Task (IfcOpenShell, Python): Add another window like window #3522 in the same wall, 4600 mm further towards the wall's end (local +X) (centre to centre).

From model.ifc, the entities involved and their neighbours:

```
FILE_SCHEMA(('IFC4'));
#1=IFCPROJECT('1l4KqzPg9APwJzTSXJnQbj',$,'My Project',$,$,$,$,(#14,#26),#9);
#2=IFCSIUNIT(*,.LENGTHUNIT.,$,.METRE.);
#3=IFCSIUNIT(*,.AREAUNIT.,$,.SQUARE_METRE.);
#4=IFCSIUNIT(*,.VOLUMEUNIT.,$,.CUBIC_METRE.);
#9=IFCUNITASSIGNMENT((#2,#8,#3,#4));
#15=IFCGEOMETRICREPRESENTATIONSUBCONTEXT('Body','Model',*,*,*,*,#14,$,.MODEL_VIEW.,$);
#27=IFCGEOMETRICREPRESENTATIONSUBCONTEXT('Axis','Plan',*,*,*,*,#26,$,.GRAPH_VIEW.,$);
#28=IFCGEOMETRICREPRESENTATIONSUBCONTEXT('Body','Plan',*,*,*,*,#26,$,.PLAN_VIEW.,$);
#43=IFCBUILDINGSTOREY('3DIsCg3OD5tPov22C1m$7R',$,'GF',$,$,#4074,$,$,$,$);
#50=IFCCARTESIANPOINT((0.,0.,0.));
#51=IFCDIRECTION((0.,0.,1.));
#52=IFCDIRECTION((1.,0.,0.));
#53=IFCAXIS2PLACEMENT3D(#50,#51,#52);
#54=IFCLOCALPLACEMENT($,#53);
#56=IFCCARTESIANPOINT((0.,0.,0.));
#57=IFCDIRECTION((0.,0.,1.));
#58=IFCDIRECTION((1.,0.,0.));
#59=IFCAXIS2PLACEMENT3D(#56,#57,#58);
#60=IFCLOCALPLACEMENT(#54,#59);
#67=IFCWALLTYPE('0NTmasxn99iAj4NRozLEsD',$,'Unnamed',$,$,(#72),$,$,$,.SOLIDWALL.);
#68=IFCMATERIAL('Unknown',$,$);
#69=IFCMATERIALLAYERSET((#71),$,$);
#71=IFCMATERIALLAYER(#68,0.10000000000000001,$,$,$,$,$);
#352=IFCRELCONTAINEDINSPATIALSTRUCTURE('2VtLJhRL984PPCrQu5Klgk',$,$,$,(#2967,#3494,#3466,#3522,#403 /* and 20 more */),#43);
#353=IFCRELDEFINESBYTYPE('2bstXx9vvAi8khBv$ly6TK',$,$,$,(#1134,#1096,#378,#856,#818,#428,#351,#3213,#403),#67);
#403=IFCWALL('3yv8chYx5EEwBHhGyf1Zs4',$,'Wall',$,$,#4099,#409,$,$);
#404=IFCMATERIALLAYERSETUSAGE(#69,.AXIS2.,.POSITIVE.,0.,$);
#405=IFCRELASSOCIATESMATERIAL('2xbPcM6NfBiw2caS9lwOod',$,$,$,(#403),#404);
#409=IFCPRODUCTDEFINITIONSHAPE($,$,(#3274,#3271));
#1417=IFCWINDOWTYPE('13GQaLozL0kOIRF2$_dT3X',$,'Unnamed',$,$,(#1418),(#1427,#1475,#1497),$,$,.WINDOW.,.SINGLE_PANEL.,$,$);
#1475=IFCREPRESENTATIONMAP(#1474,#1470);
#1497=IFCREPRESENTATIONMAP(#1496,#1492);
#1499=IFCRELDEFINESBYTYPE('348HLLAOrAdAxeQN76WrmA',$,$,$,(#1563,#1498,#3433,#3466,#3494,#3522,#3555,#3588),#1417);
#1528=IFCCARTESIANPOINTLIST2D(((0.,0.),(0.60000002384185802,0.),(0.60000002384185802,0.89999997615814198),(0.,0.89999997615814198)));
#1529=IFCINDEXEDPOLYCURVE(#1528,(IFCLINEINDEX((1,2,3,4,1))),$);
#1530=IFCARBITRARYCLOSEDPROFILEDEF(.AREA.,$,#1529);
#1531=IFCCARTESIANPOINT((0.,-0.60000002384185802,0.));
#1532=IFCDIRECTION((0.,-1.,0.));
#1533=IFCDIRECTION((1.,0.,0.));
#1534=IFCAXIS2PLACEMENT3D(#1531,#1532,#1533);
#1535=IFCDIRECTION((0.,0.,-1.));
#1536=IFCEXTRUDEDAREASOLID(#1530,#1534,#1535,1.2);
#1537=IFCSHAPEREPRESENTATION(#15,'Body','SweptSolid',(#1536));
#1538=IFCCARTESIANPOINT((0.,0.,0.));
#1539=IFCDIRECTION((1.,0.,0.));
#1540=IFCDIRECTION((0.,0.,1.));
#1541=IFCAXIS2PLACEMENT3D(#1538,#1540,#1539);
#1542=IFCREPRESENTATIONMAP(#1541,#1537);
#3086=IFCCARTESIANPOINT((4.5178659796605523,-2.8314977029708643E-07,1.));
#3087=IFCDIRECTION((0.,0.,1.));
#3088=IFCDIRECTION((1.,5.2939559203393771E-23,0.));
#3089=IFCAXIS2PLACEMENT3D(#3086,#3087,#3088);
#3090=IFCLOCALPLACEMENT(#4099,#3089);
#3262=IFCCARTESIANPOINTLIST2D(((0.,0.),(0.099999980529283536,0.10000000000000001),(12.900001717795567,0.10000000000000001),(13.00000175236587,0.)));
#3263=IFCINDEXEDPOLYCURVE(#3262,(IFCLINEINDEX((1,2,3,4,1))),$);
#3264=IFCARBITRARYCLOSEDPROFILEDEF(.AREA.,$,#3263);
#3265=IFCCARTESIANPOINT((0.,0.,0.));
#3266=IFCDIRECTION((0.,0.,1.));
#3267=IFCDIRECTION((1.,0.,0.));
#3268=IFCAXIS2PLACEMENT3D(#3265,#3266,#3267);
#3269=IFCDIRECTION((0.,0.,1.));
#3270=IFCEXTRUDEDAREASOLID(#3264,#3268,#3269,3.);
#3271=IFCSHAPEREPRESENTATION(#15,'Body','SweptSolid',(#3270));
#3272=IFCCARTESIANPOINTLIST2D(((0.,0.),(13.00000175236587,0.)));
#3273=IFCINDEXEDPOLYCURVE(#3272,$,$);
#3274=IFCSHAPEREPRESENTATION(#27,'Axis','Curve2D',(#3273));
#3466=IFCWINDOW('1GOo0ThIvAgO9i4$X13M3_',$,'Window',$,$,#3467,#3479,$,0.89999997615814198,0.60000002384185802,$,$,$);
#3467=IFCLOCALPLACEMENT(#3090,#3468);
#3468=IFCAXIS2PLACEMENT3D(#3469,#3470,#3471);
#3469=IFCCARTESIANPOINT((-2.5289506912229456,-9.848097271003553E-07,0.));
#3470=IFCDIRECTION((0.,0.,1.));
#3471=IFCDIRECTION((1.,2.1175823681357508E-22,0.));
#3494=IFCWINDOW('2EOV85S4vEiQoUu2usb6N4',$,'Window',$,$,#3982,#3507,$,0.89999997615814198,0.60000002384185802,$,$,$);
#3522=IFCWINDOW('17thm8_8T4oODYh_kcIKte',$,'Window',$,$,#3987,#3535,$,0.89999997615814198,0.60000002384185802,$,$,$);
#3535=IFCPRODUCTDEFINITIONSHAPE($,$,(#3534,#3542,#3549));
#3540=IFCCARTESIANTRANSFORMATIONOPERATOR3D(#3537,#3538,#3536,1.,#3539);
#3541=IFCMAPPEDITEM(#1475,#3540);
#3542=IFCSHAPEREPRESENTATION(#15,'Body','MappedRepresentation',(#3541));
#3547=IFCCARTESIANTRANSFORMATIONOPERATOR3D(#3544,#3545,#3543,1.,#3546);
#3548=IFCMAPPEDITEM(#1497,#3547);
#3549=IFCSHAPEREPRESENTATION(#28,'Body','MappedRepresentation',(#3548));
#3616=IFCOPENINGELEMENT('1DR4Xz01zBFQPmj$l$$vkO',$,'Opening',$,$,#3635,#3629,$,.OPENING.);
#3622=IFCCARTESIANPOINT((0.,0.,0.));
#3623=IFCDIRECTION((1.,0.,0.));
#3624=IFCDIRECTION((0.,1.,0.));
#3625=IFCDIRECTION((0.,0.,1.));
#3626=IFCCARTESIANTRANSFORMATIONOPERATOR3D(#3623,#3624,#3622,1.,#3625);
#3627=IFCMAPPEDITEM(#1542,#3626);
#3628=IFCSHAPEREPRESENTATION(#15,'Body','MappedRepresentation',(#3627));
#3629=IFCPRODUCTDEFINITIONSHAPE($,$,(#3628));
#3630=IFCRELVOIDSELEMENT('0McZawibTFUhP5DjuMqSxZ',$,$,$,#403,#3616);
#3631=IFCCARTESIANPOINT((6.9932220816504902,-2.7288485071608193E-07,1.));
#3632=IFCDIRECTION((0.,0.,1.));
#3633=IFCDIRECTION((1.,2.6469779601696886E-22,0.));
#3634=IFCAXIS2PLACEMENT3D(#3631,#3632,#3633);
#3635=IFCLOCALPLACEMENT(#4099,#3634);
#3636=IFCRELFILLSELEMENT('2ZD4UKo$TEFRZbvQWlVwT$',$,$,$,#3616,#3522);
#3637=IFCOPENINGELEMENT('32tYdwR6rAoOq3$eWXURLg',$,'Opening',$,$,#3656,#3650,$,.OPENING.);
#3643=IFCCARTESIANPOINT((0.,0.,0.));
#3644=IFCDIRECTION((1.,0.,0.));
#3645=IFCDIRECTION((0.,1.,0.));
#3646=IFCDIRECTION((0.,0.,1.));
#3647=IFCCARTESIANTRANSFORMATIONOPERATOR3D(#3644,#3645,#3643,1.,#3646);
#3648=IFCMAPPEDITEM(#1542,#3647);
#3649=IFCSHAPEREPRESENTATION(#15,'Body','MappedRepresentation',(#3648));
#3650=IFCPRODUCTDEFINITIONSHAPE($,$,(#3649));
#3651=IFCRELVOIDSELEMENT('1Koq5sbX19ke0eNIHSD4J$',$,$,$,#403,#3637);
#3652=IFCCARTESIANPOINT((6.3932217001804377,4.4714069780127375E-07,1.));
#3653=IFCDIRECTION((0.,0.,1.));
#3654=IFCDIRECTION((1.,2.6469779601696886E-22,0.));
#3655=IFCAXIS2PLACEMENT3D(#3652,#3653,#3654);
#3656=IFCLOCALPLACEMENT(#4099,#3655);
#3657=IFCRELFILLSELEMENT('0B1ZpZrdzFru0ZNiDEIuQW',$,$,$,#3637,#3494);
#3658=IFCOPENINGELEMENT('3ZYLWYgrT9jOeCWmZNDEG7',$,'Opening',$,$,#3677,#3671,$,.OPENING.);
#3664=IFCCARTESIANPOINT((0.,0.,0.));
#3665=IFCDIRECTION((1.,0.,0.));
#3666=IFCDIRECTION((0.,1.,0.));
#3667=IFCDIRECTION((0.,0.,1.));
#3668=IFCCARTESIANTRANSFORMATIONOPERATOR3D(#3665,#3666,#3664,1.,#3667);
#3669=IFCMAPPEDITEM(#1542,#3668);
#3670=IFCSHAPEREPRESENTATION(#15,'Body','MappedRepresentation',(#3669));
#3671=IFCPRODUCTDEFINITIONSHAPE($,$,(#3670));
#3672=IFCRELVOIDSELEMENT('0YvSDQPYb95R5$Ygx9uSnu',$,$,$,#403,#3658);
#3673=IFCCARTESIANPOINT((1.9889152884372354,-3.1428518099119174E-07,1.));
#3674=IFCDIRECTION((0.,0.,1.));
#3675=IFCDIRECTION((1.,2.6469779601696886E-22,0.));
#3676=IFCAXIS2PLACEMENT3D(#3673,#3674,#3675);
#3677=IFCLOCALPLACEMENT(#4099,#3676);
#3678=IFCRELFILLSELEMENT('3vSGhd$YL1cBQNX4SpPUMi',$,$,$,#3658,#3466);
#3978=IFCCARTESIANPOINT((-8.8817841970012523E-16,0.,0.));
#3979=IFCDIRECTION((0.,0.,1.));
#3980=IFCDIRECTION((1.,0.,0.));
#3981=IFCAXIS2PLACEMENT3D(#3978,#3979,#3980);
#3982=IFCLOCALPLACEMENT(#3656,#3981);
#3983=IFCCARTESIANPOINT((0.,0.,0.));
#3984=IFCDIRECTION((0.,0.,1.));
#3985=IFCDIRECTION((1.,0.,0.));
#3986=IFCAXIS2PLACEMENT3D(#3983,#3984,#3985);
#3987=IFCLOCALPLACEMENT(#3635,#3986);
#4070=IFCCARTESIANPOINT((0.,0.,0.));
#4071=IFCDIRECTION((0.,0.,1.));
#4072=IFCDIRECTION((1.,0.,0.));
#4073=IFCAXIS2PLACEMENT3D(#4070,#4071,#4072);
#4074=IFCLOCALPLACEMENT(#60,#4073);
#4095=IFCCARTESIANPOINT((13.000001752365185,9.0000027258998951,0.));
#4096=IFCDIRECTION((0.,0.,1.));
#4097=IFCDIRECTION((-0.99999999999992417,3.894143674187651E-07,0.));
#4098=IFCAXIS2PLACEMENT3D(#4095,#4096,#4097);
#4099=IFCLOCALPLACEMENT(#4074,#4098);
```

```python
import ifcopenshell
import ifcopenshell.api.feature
import ifcopenshell.api.geometry
import ifcopenshell.api.root
import ifcopenshell.geom
import ifcopenshell.util.element
import ifcopenshell.util.placement
import ifcopenshell.util.shape
import ifcopenshell.util.unit

model = ifcopenshell.open("model.ifc")
unit_scale = ifcopenshell.util.unit.calculate_unit_scale(model)
settings = ifcopenshell.geom.settings()


def volume(element):
    """Net volume in cubic metres, openings subtracted."""
    shape = ifcopenshell.geom.create_shape(settings, element)
    return ifcopenshell.util.shape.get_volume(shape.geometry)


window = model.by_guid("17thm8_8T4oODYh_kcIKte")
opening = window.FillsVoids[0].RelatingOpeningElement
wall = opening.VoidsElements[0].RelatingBuildingElement
before = volume(wall)
shift = ifcopenshell.util.placement.get_local_placement(wall.ObjectPlacement)[:3, 0] * 4.6 / unit_scale

# copy_class copies the void relationship, type, container and properties, but no geometry.
new_opening = ifcopenshell.api.root.copy_class(model, product=opening)
new_opening.Representation = ifcopenshell.util.element.copy_deep(
    model, opening.Representation, exclude=["IfcGeometricRepresentationContext", "IfcRepresentationMap"]
)
new_window = ifcopenshell.api.root.copy_class(model, product=window)
new_window.Representation = ifcopenshell.util.element.copy_deep(
    model, window.Representation, exclude=["IfcGeometricRepresentationContext", "IfcRepresentationMap"]
)
ifcopenshell.api.feature.add_filling(model, opening=new_opening, element=new_window)

for old, new in ((opening, new_opening), (window, new_window)):
    matrix = ifcopenshell.util.placement.get_local_placement(old.ObjectPlacement)
    matrix[:3, 3] += shift
    ifcopenshell.api.geometry.edit_object_placement(model, product=new, matrix=matrix, is_si=False)

after = volume(wall)

print(f"wall volume {before:.3f} -> {after:.3f} m3")

model.write("model_edited.ifc")
```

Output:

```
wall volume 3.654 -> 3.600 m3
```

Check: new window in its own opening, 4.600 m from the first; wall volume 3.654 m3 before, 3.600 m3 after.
